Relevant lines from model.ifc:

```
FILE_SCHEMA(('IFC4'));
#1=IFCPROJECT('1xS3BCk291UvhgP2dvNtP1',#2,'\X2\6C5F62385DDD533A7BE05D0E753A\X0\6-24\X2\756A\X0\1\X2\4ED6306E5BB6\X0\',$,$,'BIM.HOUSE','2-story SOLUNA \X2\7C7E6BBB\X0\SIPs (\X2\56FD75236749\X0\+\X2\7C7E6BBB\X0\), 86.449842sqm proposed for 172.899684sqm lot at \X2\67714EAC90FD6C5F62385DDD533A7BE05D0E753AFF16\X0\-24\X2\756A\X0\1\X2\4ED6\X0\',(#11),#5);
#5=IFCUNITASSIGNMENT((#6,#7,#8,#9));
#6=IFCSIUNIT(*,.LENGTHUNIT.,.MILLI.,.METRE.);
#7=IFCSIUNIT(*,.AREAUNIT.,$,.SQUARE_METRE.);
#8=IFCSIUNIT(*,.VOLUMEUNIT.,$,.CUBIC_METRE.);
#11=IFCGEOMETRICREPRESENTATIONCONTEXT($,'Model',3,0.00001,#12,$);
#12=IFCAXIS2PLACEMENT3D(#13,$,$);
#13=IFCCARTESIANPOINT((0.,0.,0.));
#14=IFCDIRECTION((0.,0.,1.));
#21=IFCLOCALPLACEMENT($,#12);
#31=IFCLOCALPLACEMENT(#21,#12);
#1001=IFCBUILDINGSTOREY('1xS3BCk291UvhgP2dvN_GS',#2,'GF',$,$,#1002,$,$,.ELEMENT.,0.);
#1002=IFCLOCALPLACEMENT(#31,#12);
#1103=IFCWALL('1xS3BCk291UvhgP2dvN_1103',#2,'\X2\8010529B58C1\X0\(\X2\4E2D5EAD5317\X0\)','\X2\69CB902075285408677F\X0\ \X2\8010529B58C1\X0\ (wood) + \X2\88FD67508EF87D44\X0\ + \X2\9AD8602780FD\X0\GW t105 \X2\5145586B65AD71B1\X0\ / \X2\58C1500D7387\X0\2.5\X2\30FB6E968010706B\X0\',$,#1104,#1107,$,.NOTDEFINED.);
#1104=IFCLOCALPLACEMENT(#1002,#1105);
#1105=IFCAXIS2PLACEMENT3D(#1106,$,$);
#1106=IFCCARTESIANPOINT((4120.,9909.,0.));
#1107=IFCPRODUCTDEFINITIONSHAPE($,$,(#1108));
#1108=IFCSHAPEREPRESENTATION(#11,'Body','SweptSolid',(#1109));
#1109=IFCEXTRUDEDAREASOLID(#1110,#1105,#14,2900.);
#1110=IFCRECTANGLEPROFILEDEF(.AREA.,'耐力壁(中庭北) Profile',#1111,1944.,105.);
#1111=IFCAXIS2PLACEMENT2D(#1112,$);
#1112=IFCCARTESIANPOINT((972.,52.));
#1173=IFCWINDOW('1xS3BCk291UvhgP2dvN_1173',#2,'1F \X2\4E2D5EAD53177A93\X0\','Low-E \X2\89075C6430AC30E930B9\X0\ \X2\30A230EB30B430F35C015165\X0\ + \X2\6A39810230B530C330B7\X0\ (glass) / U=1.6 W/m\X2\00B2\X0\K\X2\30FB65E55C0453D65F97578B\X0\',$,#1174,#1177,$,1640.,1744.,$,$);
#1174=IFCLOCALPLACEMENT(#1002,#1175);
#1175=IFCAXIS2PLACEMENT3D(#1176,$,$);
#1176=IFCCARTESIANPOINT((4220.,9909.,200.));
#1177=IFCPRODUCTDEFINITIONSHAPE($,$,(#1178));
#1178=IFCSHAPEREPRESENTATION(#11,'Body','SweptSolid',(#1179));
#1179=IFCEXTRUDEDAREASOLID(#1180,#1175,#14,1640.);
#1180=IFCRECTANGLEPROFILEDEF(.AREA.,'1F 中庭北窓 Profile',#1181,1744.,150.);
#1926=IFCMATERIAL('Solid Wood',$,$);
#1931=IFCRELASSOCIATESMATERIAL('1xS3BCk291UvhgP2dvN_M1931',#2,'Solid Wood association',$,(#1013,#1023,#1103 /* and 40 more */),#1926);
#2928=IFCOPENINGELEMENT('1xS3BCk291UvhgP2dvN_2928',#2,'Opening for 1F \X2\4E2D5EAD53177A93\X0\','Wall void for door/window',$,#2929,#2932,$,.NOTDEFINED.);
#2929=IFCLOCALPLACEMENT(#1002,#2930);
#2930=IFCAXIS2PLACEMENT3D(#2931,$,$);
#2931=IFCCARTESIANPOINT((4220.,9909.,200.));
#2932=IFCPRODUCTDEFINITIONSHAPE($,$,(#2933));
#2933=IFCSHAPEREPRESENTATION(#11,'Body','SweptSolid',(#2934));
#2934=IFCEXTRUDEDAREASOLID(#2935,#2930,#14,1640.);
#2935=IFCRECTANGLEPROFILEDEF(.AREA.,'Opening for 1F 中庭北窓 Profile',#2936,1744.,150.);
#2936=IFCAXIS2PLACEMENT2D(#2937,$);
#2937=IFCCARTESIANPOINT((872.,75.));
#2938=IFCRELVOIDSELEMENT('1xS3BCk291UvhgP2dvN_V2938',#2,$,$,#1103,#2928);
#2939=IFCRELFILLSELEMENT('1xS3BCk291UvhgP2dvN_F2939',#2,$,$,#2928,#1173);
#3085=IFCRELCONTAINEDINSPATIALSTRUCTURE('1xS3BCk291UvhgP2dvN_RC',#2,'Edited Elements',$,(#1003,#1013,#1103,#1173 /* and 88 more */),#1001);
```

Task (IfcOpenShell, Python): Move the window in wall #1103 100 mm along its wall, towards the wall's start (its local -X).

```python
import ifcopenshell
import ifcopenshell.api.geometry
import ifcopenshell.util.placement
import ifcopenshell.util.unit

model = ifcopenshell.open("model.ifc")
unit_scale = ifcopenshell.util.unit.calculate_unit_scale(model)

window = model.by_guid("1xS3BCk291UvhgP2dvN_1173")
opening = window.FillsVoids[0].RelatingOpeningElement
wall = opening.VoidsElements[0].RelatingBuildingElement

wall_matrix = ifcopenshell.util.placement.get_local_placement(wall.ObjectPlacement)
shift = wall_matrix[:3, 0] * -0.1 / unit_scale
before = ifcopenshell.util.placement.get_local_placement(window.ObjectPlacement)[:3, 3].copy()

# The window is not placed relative to its opening, so move both.
for product in (opening, window):
    matrix = ifcopenshell.util.placement.get_local_placement(product.ObjectPlacement)
    matrix[:3, 3] += shift
    ifcopenshell.api.geometry.edit_object_placement(model, product=product, matrix=matrix, is_si=False)

after = ifcopenshell.util.placement.get_local_placement(window.ObjectPlacement)[:3, 3]
print("window moved by", (after - before).round(3) + 0.0)

model.write("model_edited.ifc")
```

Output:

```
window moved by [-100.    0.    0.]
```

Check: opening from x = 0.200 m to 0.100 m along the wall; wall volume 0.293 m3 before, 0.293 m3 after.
